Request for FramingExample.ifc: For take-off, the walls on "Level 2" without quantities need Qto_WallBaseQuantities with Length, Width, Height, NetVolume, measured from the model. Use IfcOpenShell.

First a look at what the model holds.

```python
import ifcopenshell
import ifcopenshell.util.element
import ifcopenshell.util.unit

model = ifcopenshell.open("FramingExample.ifc")
print(model.schema)
for unit_type in ("LENGTHUNIT", "AREAUNIT", "VOLUMEUNIT"):
    print(unit_type, ifcopenshell.util.unit.calculate_unit_scale(model, unit_type))
storey = next(s for s in model.by_type("IfcBuildingStorey") if s.Name == "Level 2")
walls = [e for e in ifcopenshell.util.element.get_decomposition(storey) if e.is_a("IfcWall")]
for e in sorted(walls, key=lambda e: e.id()):
    print(e.id(), e.is_a(), e.Name, list(ifcopenshell.util.element.get_psets(e, qtos_only=True)), sep=" | ")
```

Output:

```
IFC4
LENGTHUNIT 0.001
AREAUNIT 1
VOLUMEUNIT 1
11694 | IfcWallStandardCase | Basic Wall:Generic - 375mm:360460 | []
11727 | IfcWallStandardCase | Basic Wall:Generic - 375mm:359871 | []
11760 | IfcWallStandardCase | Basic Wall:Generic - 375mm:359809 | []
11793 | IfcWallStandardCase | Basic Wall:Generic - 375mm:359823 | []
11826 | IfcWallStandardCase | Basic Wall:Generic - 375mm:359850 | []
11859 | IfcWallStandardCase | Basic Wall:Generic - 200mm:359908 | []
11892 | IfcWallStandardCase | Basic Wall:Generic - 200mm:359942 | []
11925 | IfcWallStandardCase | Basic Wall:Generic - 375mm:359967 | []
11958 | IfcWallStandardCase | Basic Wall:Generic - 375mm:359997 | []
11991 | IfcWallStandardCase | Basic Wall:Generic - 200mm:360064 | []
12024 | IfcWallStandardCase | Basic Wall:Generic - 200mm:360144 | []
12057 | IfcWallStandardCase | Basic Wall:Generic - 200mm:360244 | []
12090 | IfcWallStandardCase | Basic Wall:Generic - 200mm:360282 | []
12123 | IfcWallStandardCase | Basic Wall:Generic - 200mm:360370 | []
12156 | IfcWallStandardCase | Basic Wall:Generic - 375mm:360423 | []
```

```python
import ifcopenshell
import ifcopenshell.api.pset
import ifcopenshell.geom
import ifcopenshell.util.element
import ifcopenshell.util.shape
import ifcopenshell.util.unit

model = ifcopenshell.open("FramingExample.ifc")
unit_scale = ifcopenshell.util.unit.calculate_unit_scale(model)
volume_scale = ifcopenshell.util.unit.calculate_unit_scale(model, "VOLUMEUNIT")
settings = ifcopenshell.geom.settings()

storey = next(s for s in model.by_type("IfcBuildingStorey") if s.Name == "Level 2")
walls = [e for e in ifcopenshell.util.element.get_decomposition(storey) if e.is_a("IfcWall")]

for e in sorted(walls, key=lambda e: e.id()):
    if ifcopenshell.util.element.get_psets(e, qtos_only=True, should_inherit=False):
        continue
    # Geometry comes back in metres, in the element's own axes.
    shape = ifcopenshell.geom.create_shape(settings, e)
    values = {
        "Length": ifcopenshell.util.shape.get_x(shape.geometry) / unit_scale,
        "Width": ifcopenshell.util.shape.get_y(shape.geometry) / unit_scale,
        "Height": ifcopenshell.util.shape.get_z(shape.geometry) / unit_scale,
        "NetVolume": ifcopenshell.util.shape.get_volume(shape.geometry) / volume_scale,
    }
    qto = ifcopenshell.api.pset.add_qto(model, product=e, name="Qto_WallBaseQuantities")
    ifcopenshell.api.pset.edit_qto(model, qto=qto, properties=values)
    print(e.id(), {k: round(v, 3) for k, v in values.items()})

model.write("FramingExample_rev.ifc")
```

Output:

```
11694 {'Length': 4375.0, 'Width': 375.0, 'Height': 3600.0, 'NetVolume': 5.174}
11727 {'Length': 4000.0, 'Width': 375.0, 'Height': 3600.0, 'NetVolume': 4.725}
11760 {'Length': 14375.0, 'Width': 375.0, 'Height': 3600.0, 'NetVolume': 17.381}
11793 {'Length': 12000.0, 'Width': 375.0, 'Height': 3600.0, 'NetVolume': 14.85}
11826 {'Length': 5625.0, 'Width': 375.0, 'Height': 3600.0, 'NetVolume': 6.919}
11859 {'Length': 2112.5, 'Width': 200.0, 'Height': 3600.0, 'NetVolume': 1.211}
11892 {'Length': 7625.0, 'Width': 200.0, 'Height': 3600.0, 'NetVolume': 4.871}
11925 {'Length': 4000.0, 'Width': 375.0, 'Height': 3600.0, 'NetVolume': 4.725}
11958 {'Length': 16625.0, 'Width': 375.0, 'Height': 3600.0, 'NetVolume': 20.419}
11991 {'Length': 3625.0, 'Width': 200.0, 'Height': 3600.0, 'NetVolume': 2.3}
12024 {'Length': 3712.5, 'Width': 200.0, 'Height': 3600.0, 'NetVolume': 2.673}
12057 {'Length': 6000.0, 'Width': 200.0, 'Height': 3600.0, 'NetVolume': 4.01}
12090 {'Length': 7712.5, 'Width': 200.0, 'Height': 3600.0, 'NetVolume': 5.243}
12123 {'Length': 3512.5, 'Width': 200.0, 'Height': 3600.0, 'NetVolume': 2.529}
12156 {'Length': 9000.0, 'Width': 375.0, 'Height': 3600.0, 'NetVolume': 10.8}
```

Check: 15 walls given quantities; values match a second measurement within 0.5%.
